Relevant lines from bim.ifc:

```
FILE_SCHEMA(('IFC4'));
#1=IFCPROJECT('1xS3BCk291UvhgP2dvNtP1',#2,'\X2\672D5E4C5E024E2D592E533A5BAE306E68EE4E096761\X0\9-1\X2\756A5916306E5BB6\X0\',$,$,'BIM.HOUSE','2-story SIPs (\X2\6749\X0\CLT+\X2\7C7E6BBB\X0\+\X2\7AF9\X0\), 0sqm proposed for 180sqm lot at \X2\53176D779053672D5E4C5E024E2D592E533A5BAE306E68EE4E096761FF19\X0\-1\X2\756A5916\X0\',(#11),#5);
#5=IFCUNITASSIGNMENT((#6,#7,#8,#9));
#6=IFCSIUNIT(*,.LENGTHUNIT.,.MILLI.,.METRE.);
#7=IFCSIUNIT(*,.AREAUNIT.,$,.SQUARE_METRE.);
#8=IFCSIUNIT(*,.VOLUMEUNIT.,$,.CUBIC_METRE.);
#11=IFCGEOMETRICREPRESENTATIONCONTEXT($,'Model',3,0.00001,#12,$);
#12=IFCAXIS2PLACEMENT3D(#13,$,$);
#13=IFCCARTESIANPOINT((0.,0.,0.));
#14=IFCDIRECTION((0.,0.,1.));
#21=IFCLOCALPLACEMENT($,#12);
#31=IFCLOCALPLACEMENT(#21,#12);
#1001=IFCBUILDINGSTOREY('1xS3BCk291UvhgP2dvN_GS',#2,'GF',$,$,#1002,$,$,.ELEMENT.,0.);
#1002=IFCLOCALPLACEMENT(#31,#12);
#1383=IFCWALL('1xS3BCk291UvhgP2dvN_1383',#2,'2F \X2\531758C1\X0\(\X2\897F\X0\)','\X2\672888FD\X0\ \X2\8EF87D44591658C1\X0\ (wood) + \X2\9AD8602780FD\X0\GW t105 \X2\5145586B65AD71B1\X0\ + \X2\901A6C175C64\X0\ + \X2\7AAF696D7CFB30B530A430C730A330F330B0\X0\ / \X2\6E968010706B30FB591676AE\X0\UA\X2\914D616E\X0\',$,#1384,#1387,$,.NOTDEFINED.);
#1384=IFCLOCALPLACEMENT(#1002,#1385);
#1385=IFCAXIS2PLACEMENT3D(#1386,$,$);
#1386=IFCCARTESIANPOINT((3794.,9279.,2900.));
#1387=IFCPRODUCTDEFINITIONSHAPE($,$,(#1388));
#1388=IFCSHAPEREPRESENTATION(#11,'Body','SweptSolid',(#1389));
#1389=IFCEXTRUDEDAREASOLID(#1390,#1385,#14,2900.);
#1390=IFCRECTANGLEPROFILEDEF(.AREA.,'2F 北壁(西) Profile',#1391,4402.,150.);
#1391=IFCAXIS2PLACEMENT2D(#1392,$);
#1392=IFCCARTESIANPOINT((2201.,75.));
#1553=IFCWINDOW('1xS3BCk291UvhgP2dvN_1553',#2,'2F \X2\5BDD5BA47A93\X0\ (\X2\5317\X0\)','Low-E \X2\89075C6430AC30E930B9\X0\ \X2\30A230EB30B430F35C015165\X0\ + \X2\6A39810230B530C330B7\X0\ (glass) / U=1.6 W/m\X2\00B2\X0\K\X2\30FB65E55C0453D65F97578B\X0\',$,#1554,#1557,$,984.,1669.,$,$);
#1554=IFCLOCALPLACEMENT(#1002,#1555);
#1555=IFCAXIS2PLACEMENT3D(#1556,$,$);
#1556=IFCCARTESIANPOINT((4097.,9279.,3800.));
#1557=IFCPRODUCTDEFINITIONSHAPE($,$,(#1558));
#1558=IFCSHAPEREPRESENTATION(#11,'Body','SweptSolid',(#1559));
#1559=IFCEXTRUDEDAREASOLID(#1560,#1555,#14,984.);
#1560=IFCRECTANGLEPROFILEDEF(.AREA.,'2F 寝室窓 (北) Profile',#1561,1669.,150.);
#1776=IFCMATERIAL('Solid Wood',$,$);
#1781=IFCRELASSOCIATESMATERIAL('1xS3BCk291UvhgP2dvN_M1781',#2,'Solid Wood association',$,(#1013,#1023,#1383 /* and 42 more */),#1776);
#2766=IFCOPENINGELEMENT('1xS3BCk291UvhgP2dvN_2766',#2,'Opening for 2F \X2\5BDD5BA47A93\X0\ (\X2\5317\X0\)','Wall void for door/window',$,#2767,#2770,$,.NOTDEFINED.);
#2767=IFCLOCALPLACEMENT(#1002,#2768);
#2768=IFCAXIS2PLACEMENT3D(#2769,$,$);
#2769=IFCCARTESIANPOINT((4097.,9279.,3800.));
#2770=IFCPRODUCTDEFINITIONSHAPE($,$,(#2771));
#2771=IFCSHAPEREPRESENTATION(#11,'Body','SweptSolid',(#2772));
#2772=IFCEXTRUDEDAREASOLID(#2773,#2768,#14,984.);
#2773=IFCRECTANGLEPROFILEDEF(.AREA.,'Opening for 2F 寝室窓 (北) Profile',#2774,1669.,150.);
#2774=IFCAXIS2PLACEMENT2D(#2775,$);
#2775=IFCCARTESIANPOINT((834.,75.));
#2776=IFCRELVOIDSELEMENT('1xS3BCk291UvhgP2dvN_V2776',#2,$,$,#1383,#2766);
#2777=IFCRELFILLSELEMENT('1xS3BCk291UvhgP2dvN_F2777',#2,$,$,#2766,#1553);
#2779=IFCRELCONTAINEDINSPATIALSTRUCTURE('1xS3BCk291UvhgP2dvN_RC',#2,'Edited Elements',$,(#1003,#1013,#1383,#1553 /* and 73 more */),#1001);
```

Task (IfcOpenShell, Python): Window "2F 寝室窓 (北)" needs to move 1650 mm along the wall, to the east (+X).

```python
import ifcopenshell
import ifcopenshell.api.geometry
import ifcopenshell.util.placement

model = ifcopenshell.open("bim.ifc")

window = model.by_guid("1xS3BCk291UvhgP2dvN_1553")
opening = window.FillsVoids[0].RelatingOpeningElement
wall = opening.VoidsElements[0].RelatingBuildingElement

wall_matrix = ifcopenshell.util.placement.get_local_placement(wall.ObjectPlacement)
shift = wall_matrix[:3, 0] * 1650.0
before = ifcopenshell.util.placement.get_local_placement(window.ObjectPlacement)[:3, 3].copy()

# The window is not placed relative to its opening, so move both.
for product in (opening, window):
    matrix = ifcopenshell.util.placement.get_local_placement(product.ObjectPlacement)
    matrix[:3, 3] += shift
    ifcopenshell.api.geometry.edit_object_placement(model, product=product, matrix=matrix, is_si=False)

after = ifcopenshell.util.placement.get_local_placement(window.ObjectPlacement)[:3, 3]
print("window moved by", (after - before).round(3) + 0.0)

model.write("bim_rev.ifc")
```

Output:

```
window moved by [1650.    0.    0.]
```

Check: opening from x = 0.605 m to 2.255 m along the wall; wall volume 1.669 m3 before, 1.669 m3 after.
